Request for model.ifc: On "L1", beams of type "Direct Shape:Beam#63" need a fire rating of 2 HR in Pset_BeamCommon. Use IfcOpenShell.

First a look at what the model holds.

```python
import ifcopenshell
import ifcopenshell.util.element

model = ifcopenshell.open("model.ifc")
print(model.schema)
storey = next(s for s in model.by_type("IfcBuildingStorey") if s.Name == "L1")
beams = [e for e in ifcopenshell.util.element.get_decomposition(storey) if e.is_a("IfcBeam")]
seen = {}
for e in beams:
    element_type = ifcopenshell.util.element.get_type(e)
    key = (element_type.Name if element_type != e and element_type else None, ifcopenshell.util.element.get_pset(e, "Pset_BeamCommon", "FireRating"))
    seen[key] = seen.get(key, 0) + 1
for (name, value), count in sorted(seen.items(), key=str):
    print(count, "x", name, "|", value)
```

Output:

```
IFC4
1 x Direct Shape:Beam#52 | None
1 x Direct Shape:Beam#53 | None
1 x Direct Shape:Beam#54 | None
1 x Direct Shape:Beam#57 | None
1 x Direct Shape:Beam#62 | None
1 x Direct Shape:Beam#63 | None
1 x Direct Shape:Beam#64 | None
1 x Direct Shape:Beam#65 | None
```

```python
import ifcopenshell
import ifcopenshell.api.pset
import ifcopenshell.util.element

model = ifcopenshell.open("model.ifc")

storey = next(s for s in model.by_type("IfcBuildingStorey") if s.Name == "L1")
beams = [e for e in ifcopenshell.util.element.get_decomposition(storey) if e.is_a("IfcBeam")]

count = 0
for e in beams:
    element_type = ifcopenshell.util.element.get_type(e)
    if element_type in (None, e) or element_type.Name != "Direct Shape:Beam#63":
        continue
    # add_pset returns the element's existing set when there is one.
    pset = ifcopenshell.api.pset.add_pset(model, product=e, name="Pset_BeamCommon")
    ifcopenshell.api.pset.edit_pset(model, pset=pset, properties={"FireRating": "2 HR"})
    count += 1

print(count, "beams updated")

model.write("model_rev.ifc")
```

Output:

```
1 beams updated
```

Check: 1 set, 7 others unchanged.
